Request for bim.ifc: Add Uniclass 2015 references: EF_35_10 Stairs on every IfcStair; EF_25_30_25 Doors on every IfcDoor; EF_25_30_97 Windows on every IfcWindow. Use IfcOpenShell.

First a look at what the model holds.

```python
import ifcopenshell

model = ifcopenshell.open("bim.ifc")
print(model.schema)
print("classifications:", [c.Name for c in model.by_type("IfcClassification")])
for ifc_class in ("IfcDoor", "IfcRoof", "IfcStair", "IfcWall", "IfcWindow"):
    print(ifc_class, len(model.by_type(ifc_class)))
```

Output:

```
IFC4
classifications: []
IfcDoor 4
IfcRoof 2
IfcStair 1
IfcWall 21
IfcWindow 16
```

```python
import ifcopenshell
import ifcopenshell.api.classification

model = ifcopenshell.open("bim.ifc")

system = ifcopenshell.api.classification.add_classification(model, classification="Uniclass 2015")

codes = {
    "IfcStair": ("EF_35_10", "Stairs"),
    "IfcDoor": ("EF_25_30_25", "Doors"),
    "IfcWindow": ("EF_25_30_97", "Windows"),
}
for ifc_class, (code, name) in codes.items():
    products = model.by_type(ifc_class)
    ifcopenshell.api.classification.add_reference(
        model, products=products, classification=system, identification=code, name=name
    )
    print(code, len(products))

model.write("bim-out.ifc")
```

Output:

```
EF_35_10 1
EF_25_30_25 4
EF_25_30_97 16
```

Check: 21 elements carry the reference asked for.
